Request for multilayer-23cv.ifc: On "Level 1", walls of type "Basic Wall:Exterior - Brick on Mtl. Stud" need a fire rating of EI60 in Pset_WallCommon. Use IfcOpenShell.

First a look at what the model holds.

```python
import ifcopenshell
import ifcopenshell.util.element

model = ifcopenshell.open("multilayer-23cv.ifc")
print(model.schema)
storey = next(s for s in model.by_type("IfcBuildingStorey") if s.Name == "Level 1")
walls = [e for e in ifcopenshell.util.element.get_decomposition(storey) if e.is_a("IfcWall")]
seen = {}
for e in walls:
    element_type = ifcopenshell.util.element.get_type(e)
    key = (element_type.Name if element_type != e and element_type else None, ifcopenshell.util.element.get_pset(e, "Pset_WallCommon", "FireRating"))
    seen[key] = seen.get(key, 0) + 1
for (name, value), count in sorted(seen.items(), key=str):
    print(count, "x", name, "|", value)
```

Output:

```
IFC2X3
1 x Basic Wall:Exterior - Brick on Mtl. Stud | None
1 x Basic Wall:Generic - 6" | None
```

```python
import ifcopenshell
import ifcopenshell.api.pset
import ifcopenshell.util.element

model = ifcopenshell.open("multilayer-23cv.ifc")

storey = next(s for s in model.by_type("IfcBuildingStorey") if s.Name == "Level 1")
walls = [e for e in ifcopenshell.util.element.get_decomposition(storey) if e.is_a("IfcWall")]

count = 0
for e in walls:
    element_type = ifcopenshell.util.element.get_type(e)
    if element_type in (None, e) or element_type.Name != "Basic Wall:Exterior - Brick on Mtl. Stud":
        continue
    # add_pset returns the element's existing set when there is one.
    pset = ifcopenshell.api.pset.add_pset(model, product=e, name="Pset_WallCommon")
    ifcopenshell.api.pset.edit_pset(model, pset=pset, properties={"FireRating": "EI60"})
    count += 1

print(count, "walls updated")

model.write("multilayer-23cv_edited.ifc")
```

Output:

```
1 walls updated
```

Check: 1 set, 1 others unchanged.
